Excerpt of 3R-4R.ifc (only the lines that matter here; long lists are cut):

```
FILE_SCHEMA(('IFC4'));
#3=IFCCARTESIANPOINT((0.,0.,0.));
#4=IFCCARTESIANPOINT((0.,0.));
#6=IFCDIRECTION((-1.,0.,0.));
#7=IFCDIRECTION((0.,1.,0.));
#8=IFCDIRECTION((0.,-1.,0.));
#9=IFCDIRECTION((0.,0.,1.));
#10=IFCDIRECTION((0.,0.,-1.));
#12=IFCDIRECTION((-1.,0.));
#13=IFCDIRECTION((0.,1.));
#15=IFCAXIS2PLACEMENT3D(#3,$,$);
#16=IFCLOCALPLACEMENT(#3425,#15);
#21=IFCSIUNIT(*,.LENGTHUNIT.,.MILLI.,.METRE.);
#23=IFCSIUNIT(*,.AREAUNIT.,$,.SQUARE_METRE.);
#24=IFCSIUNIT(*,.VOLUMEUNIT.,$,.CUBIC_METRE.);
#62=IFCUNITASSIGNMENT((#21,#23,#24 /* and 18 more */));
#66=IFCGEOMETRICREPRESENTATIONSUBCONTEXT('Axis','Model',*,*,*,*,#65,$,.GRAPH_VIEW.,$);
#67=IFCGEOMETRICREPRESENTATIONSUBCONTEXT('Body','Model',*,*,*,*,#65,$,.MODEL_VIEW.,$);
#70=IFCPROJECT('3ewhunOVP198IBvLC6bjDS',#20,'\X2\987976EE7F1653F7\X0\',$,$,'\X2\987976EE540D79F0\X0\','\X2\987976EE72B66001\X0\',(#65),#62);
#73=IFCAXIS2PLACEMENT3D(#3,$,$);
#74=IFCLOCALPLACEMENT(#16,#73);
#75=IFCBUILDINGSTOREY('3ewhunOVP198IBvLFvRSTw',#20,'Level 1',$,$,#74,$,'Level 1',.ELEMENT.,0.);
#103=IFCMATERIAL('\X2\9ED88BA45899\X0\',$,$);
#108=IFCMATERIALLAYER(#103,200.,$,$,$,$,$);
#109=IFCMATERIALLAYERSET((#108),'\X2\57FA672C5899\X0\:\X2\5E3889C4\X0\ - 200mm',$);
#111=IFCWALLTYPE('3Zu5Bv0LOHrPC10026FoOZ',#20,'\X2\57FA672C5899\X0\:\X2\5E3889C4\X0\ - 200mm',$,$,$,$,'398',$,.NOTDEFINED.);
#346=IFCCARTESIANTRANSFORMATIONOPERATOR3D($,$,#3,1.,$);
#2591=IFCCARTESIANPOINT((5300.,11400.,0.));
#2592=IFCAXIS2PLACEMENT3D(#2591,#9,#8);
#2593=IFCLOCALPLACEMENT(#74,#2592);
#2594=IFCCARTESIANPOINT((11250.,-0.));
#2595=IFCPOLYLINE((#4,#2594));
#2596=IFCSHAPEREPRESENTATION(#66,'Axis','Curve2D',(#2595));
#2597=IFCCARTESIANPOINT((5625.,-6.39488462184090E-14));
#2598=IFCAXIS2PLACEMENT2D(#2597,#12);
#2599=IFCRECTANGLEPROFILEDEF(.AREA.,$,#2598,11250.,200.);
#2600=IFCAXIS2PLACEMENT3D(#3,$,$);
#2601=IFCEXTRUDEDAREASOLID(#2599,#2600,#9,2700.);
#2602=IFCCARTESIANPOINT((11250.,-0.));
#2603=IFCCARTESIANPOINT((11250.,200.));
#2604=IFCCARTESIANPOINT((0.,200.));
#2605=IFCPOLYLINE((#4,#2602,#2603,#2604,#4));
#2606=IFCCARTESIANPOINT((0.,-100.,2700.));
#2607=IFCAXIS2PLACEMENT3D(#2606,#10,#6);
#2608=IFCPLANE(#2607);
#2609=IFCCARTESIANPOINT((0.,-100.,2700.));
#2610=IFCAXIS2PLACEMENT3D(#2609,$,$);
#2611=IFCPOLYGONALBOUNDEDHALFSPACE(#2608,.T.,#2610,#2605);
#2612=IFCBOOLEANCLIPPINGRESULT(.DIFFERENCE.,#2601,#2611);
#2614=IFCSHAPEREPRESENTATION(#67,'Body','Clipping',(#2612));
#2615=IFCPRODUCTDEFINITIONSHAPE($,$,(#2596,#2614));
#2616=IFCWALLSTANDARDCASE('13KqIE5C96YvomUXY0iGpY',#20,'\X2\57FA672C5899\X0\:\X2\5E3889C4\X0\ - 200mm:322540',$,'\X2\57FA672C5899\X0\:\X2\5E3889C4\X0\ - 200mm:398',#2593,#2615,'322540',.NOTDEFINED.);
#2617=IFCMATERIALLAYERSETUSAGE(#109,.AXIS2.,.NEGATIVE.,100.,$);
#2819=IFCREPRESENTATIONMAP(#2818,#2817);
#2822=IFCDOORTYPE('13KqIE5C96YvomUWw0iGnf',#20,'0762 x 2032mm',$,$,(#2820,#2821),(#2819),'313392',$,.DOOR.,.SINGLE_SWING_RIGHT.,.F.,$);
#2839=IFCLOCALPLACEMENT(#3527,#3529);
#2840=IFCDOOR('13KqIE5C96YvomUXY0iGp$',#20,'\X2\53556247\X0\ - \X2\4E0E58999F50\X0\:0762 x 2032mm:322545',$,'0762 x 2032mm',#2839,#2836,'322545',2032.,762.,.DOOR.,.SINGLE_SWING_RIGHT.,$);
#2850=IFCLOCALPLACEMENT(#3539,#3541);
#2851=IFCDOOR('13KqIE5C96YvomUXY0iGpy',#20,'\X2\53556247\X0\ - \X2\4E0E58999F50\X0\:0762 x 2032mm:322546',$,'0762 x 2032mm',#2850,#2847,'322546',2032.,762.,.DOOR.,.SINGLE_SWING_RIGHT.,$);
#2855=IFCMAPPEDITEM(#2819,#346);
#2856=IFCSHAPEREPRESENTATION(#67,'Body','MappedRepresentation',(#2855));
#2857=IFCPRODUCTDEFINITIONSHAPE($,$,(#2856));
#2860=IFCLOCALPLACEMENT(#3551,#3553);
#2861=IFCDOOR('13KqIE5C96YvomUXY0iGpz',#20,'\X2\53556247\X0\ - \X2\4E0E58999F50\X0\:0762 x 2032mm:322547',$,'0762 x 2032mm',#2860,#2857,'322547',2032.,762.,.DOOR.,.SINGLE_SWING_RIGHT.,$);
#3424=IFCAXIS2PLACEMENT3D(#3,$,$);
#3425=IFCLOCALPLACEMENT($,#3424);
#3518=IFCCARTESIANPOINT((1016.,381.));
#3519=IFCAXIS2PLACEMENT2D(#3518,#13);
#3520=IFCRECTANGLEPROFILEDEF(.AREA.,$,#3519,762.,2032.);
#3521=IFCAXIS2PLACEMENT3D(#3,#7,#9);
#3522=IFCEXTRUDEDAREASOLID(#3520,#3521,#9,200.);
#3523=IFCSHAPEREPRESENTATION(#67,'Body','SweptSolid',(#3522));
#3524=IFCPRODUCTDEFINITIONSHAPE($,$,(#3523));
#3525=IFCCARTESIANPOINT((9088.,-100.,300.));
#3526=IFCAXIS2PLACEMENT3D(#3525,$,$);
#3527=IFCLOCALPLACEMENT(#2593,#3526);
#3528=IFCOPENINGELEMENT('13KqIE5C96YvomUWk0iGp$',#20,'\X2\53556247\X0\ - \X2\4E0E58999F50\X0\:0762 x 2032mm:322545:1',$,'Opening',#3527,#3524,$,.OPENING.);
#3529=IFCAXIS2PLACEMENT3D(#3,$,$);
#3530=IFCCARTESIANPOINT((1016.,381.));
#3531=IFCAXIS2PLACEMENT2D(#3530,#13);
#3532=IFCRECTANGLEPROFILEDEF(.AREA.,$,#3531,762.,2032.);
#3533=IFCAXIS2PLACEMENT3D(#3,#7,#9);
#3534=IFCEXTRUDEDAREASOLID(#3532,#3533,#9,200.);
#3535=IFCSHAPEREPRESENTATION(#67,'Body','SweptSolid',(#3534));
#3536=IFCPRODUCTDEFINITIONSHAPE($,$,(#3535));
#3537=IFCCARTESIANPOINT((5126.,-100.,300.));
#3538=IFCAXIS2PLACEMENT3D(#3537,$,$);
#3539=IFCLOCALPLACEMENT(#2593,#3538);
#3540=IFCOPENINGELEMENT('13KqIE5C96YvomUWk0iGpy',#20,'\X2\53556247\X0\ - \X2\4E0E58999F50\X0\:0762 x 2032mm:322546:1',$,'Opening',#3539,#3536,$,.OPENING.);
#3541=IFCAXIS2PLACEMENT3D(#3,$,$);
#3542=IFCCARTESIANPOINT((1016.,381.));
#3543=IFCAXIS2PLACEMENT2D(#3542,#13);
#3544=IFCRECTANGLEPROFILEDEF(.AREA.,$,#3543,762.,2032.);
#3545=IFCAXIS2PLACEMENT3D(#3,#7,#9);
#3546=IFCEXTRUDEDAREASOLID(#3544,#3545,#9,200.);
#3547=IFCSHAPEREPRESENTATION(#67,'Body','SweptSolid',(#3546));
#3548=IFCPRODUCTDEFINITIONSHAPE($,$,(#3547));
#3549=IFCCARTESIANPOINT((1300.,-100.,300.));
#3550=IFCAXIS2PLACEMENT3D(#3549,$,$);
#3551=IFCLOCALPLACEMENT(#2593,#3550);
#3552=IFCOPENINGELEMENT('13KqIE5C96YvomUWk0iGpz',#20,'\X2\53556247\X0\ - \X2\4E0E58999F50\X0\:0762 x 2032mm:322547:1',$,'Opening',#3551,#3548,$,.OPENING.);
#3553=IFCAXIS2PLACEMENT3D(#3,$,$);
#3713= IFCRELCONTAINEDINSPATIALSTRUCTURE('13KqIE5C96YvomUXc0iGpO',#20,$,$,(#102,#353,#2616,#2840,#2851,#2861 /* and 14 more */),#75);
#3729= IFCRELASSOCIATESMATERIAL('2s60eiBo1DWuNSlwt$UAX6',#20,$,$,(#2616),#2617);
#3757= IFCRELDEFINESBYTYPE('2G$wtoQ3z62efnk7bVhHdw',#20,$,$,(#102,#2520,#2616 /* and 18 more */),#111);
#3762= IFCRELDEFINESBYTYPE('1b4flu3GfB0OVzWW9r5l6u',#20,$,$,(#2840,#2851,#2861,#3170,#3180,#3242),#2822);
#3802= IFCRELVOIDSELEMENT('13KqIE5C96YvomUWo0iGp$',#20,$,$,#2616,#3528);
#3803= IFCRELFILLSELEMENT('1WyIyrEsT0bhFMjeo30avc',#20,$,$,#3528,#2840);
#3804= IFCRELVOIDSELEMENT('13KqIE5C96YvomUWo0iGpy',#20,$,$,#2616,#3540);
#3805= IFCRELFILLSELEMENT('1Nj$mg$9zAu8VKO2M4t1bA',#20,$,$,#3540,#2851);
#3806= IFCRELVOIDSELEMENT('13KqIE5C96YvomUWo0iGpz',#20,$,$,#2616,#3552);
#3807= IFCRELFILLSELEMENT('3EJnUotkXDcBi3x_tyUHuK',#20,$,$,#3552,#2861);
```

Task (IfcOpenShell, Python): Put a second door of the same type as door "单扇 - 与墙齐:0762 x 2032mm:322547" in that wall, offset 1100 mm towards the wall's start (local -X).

```python
import ifcopenshell
import ifcopenshell.api.feature
import ifcopenshell.api.geometry
import ifcopenshell.api.root
import ifcopenshell.geom
import ifcopenshell.util.element
import ifcopenshell.util.placement
import ifcopenshell.util.shape
import ifcopenshell.util.unit

model = ifcopenshell.open("3R-4R.ifc")
unit_scale = ifcopenshell.util.unit.calculate_unit_scale(model)
settings = ifcopenshell.geom.settings()


def volume(element):
    """Net volume in cubic metres, openings subtracted."""
    shape = ifcopenshell.geom.create_shape(settings, element)
    return ifcopenshell.util.shape.get_volume(shape.geometry)


def reuse_history(source, copy):
    """copy_class also copies each property set's owner history, people and application; keep the originals."""
    for rel in copy.IsDefinedBy:
        if rel.is_a("IfcRelDefinesByProperties") and (history := rel.RelatingPropertyDefinition.OwnerHistory):
            rel.RelatingPropertyDefinition.OwnerHistory = source.OwnerHistory
            ifcopenshell.util.element.remove_deep2(model, history)


door = model.by_id(2861)
opening = door.FillsVoids[0].RelatingOpeningElement
wall = opening.VoidsElements[0].RelatingBuildingElement
before = volume(wall)
shift = ifcopenshell.util.placement.get_local_placement(wall.ObjectPlacement)[:3, 0] * -1.1 / unit_scale

# copy_class copies the void relationship, type, container and properties, but no geometry.
new_opening = ifcopenshell.api.root.copy_class(model, product=opening)
new_opening.Representation = ifcopenshell.util.element.copy_deep(
    model, opening.Representation, exclude=["IfcGeometricRepresentationContext", "IfcRepresentationMap"]
)
new_opening.Name = "单扇 - 与墙齐:0762 x 2032mm"
new_door = ifcopenshell.api.root.copy_class(model, product=door)
new_door.Representation = ifcopenshell.util.element.copy_deep(
    model, door.Representation, exclude=["IfcGeometricRepresentationContext", "IfcRepresentationMap"]
)
new_door.Name = "单扇 - 与墙齐:0762 x 2032mm"
new_door.Tag = None
reuse_history(door, new_door)
ifcopenshell.api.feature.add_filling(model, opening=new_opening, element=new_door)

for old, new in ((opening, new_opening), (door, new_door)):
    matrix = ifcopenshell.util.placement.get_local_placement(old.ObjectPlacement)
    matrix[:3, 3] += shift
    ifcopenshell.api.geometry.edit_object_placement(model, product=new, matrix=matrix, is_si=False)

after = volume(wall)

print(f"wall volume {before:.3f} -> {after:.3f} m3")

model.write("3R-4R_v2.ifc")
```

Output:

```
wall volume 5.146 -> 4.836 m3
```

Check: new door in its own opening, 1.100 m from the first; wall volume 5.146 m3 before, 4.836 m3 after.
